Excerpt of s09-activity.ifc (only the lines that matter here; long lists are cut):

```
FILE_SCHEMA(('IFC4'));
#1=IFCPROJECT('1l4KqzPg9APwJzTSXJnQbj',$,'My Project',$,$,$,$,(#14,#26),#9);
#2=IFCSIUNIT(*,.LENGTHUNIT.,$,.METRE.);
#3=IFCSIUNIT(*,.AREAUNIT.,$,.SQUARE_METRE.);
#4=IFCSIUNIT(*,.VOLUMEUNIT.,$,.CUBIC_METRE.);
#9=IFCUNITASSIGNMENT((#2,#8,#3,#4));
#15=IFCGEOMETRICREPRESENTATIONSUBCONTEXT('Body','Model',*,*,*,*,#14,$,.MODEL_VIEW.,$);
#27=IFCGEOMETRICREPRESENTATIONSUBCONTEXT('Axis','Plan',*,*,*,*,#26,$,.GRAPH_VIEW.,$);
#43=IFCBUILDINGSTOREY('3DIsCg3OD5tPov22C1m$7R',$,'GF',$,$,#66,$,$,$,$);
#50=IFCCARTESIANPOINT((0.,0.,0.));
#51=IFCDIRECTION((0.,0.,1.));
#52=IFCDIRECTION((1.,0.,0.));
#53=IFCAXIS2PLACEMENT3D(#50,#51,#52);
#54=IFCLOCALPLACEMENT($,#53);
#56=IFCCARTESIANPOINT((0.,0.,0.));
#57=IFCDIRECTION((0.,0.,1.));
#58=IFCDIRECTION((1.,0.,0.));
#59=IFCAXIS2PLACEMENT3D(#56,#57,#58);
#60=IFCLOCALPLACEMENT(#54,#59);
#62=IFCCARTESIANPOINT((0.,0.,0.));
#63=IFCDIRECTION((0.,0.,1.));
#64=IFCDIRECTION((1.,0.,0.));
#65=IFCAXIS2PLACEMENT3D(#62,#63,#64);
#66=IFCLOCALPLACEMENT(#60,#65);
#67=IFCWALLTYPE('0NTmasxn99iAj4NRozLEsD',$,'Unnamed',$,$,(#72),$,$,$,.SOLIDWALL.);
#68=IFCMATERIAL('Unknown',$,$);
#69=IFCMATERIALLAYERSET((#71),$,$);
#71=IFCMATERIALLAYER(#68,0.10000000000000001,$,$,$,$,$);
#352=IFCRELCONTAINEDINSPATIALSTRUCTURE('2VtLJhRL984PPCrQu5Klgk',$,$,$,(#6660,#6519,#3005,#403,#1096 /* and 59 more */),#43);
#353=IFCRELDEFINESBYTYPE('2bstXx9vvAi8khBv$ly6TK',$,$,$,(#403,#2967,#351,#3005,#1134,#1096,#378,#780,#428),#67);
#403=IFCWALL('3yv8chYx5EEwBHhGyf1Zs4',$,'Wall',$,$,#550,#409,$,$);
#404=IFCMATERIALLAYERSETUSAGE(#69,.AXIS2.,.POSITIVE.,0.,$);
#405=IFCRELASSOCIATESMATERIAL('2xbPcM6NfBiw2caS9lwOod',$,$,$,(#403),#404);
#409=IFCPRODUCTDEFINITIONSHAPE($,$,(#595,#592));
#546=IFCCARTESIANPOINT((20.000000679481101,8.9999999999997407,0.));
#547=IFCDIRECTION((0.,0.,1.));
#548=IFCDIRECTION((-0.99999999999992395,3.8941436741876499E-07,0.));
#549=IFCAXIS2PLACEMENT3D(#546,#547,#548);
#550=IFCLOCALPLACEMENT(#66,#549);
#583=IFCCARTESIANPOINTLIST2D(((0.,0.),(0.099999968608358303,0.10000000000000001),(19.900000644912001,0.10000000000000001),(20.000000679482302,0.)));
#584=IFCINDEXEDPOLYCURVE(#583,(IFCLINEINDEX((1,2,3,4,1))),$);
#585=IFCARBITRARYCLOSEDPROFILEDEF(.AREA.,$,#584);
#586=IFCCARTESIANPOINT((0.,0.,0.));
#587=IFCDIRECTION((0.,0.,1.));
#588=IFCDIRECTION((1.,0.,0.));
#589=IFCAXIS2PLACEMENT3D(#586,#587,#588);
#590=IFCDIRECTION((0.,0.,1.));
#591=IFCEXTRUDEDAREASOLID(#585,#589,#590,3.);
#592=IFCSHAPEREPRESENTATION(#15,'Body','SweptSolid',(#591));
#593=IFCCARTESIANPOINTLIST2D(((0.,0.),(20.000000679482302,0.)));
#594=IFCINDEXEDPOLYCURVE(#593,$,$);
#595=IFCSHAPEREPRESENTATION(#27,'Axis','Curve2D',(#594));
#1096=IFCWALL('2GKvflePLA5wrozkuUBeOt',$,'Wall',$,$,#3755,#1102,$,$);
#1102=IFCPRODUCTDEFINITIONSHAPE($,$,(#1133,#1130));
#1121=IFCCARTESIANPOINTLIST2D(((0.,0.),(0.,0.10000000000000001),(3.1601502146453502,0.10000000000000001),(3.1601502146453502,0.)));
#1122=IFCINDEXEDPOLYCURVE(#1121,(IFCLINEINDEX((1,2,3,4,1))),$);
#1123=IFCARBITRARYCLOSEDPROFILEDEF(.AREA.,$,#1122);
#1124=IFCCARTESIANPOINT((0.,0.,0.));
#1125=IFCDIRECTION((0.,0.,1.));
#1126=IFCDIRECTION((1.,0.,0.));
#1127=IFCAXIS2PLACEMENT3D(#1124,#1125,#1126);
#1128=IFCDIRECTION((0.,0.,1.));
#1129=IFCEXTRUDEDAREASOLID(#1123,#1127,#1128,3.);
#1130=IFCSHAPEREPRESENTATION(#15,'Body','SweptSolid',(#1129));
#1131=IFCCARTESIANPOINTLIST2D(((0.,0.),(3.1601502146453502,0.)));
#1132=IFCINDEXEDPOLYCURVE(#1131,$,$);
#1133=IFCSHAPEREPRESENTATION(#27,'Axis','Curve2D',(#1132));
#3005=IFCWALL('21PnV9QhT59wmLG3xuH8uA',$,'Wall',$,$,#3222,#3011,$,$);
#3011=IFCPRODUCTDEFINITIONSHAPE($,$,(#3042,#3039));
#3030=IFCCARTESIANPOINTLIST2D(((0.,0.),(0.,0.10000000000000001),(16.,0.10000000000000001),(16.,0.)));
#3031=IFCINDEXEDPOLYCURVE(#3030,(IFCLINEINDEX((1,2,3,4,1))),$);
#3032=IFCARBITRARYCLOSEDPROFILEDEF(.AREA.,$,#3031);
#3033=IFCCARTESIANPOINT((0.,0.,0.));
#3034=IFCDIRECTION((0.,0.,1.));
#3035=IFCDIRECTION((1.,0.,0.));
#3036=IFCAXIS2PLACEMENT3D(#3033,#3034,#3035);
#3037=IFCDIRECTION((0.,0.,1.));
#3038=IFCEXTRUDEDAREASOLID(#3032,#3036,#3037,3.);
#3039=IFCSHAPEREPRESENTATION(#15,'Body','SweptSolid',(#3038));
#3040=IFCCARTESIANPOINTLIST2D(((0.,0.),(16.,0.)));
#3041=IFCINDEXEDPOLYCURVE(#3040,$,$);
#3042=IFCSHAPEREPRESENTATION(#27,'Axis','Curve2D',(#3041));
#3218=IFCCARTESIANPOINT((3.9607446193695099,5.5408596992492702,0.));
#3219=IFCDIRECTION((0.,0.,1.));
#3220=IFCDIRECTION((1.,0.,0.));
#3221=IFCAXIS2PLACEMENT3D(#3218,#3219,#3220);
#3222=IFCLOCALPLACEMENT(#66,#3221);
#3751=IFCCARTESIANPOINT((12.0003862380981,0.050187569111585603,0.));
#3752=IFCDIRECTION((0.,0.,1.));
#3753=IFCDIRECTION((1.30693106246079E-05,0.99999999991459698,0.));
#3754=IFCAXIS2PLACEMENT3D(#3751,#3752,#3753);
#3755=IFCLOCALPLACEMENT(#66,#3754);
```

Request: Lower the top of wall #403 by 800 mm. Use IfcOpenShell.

```python
import ifcopenshell
import ifcopenshell.geom
import ifcopenshell.util.representation
import ifcopenshell.util.shape

model = ifcopenshell.open("s09-activity.ifc")
settings = ifcopenshell.geom.settings()


def volume(element):
    """Net volume in cubic metres, openings subtracted."""
    shape = ifcopenshell.geom.create_shape(settings, element)
    return ifcopenshell.util.shape.get_volume(shape.geometry)


wall = model.by_guid("3yv8chYx5EEwBHhGyf1Zs4")
before = volume(wall)

body = ifcopenshell.util.representation.get_representation(wall, "Model", "Body")
solid = body.Items[0]
old_height = solid.Depth
solid.Depth -= 0.8
after = volume(wall)

print(f"height {old_height:g} -> {solid.Depth:g}, volume {before:.3f} -> {after:.3f} m3")

model.write("s09-activity_updated.ifc")
```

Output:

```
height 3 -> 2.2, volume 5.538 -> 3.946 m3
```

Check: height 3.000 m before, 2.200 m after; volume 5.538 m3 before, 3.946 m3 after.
